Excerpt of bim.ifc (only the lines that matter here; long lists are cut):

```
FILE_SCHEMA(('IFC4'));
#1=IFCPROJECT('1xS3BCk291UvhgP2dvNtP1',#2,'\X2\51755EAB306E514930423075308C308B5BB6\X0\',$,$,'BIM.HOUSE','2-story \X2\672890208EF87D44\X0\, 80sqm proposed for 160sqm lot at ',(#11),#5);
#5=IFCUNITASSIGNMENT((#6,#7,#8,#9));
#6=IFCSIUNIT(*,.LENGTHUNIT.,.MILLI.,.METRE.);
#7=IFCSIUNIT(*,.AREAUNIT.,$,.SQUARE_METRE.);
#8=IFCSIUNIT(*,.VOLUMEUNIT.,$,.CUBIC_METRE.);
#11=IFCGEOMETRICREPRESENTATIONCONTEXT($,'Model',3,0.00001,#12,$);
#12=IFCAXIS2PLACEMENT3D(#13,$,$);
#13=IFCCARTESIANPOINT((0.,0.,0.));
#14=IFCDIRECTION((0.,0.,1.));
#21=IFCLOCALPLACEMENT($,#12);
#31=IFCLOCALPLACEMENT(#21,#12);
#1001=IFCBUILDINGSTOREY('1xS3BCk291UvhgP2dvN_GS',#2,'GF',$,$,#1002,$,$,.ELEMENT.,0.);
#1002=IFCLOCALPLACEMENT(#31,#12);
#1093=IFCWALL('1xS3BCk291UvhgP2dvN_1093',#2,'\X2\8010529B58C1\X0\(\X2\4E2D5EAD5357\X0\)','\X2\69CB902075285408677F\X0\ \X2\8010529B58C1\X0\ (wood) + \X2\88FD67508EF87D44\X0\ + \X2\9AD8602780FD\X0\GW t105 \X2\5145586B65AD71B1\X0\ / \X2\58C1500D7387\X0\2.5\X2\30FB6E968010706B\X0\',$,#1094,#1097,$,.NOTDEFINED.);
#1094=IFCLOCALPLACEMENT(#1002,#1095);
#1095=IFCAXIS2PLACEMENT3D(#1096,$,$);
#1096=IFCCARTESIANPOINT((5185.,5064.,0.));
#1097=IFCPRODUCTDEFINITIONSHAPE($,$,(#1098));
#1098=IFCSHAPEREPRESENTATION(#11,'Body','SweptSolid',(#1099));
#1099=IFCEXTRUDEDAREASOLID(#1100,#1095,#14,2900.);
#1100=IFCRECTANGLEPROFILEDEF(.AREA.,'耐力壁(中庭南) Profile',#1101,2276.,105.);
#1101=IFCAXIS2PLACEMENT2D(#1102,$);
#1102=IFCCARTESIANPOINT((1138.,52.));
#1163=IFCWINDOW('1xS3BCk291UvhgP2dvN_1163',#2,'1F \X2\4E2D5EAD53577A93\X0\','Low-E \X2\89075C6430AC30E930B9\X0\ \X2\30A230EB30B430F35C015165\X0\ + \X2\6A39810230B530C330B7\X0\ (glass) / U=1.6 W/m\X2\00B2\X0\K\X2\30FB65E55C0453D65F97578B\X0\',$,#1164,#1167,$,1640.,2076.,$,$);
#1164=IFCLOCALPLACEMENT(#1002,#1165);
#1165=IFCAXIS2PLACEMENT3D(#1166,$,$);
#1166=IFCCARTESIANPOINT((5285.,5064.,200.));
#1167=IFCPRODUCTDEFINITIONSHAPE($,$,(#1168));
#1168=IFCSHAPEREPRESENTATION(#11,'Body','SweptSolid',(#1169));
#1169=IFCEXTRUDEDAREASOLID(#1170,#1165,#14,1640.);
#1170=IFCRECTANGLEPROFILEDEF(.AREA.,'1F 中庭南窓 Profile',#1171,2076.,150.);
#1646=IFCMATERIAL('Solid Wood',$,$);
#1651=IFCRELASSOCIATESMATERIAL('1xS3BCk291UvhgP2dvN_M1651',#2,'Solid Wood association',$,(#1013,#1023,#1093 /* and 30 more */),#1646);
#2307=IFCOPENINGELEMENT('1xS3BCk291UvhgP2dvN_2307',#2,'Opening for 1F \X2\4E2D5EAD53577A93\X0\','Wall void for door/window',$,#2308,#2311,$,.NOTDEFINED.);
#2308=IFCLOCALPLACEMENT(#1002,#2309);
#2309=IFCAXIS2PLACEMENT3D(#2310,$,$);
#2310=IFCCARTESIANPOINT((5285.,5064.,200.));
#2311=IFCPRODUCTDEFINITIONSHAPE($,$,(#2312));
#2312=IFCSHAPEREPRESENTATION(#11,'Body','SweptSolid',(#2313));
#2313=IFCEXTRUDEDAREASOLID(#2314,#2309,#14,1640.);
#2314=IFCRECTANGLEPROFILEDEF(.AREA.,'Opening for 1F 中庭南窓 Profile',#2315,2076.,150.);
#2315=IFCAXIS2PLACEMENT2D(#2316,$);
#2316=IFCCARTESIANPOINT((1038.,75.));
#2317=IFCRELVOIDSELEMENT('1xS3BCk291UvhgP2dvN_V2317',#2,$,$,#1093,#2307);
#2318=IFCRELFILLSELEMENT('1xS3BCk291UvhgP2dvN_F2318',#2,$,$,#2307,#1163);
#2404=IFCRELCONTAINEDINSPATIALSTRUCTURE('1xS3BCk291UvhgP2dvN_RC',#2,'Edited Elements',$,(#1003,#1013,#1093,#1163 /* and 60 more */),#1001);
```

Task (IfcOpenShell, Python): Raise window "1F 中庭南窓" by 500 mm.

```python
import numpy as np
import ifcopenshell
import ifcopenshell.api.geometry
import ifcopenshell.util.placement
import ifcopenshell.util.unit

model = ifcopenshell.open("bim.ifc")
unit_scale = ifcopenshell.util.unit.calculate_unit_scale(model)

window = model.by_id(1163)
opening = window.FillsVoids[0].RelatingOpeningElement
dz = 0.5 / unit_scale

shift = np.array([0.0, 0.0, dz])
# The window is not placed relative to its opening, so move both.
for product in (opening, window):
    matrix = ifcopenshell.util.placement.get_local_placement(product.ObjectPlacement)
    matrix[:3, 3] += shift
    ifcopenshell.api.geometry.edit_object_placement(model, product=product, matrix=matrix, is_si=False)

print(f"moved by {dz * unit_scale:+.3f} m")

model.write("bim_edited.ifc")
```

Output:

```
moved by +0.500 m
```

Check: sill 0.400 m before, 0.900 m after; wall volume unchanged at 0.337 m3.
